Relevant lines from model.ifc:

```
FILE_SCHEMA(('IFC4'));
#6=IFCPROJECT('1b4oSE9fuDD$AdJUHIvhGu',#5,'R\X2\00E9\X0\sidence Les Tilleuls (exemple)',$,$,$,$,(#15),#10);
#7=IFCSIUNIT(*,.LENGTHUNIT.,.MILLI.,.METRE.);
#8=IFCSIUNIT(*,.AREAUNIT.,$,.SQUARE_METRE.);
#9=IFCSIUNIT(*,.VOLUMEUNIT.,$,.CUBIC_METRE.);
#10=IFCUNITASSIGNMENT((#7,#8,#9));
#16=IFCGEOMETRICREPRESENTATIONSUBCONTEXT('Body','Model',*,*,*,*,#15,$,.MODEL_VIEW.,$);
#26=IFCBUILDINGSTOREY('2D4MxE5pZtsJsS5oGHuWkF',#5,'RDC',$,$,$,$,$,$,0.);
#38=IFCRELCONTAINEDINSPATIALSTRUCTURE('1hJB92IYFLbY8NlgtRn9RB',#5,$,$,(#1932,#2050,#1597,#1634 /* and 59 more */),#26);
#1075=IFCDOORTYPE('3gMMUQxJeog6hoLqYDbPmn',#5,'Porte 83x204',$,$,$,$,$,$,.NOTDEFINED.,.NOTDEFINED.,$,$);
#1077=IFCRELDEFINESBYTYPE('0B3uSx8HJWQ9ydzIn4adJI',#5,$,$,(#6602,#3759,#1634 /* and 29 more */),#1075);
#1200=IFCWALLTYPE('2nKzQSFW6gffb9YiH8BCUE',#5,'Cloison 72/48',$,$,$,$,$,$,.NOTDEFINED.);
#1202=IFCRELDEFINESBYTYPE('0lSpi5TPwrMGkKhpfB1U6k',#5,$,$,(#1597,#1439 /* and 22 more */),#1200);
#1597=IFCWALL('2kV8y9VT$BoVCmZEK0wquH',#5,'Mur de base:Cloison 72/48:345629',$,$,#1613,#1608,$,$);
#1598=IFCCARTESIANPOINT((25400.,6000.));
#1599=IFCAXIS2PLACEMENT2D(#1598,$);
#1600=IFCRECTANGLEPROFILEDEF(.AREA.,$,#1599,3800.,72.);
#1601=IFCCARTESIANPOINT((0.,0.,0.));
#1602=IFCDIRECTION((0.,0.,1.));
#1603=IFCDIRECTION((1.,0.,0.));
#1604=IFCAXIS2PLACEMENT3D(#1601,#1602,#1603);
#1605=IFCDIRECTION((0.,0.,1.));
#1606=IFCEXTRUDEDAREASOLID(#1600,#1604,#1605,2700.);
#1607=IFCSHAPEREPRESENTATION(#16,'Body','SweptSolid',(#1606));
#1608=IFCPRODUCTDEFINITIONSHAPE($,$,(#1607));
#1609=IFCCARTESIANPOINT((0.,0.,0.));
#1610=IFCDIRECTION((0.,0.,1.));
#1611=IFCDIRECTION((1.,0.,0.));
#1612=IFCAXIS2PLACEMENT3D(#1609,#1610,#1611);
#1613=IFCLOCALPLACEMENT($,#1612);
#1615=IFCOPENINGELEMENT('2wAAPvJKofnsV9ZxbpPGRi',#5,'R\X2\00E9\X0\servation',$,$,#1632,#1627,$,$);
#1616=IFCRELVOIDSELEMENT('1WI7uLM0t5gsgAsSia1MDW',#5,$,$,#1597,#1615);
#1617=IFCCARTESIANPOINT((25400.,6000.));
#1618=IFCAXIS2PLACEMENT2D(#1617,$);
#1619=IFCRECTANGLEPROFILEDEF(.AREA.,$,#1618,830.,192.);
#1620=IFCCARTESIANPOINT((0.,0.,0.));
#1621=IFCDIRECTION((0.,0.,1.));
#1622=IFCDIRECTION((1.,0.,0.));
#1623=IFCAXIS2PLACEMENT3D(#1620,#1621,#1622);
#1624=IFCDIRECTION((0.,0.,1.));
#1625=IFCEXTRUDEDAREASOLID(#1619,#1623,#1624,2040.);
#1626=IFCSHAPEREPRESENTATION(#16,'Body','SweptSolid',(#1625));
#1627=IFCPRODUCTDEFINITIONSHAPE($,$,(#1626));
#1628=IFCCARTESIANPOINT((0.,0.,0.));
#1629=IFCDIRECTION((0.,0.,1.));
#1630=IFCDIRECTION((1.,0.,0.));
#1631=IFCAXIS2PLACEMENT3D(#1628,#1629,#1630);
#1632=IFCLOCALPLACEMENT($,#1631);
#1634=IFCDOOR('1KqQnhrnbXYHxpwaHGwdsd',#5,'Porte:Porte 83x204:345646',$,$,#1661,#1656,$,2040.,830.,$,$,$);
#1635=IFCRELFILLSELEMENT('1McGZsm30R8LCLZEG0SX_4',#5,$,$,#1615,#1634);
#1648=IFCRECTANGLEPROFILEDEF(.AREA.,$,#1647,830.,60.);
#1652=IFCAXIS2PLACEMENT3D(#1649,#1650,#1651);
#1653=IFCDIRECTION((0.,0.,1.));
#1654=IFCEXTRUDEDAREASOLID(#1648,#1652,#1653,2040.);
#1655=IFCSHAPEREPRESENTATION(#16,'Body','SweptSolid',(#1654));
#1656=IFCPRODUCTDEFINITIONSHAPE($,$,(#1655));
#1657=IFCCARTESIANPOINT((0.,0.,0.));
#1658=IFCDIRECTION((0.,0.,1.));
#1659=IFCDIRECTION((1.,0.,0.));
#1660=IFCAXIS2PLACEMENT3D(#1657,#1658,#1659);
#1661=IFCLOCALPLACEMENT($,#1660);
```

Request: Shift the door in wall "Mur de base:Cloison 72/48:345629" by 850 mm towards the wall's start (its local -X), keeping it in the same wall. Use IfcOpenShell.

```python
import ifcopenshell
import ifcopenshell.api.geometry
import ifcopenshell.util.placement
import ifcopenshell.util.unit

model = ifcopenshell.open("model.ifc")
unit_scale = ifcopenshell.util.unit.calculate_unit_scale(model)

door = model.by_id(1634)
opening = door.FillsVoids[0].RelatingOpeningElement
wall = opening.VoidsElements[0].RelatingBuildingElement

wall_matrix = ifcopenshell.util.placement.get_local_placement(wall.ObjectPlacement)
shift = wall_matrix[:3, 0] * -0.85 / unit_scale
before = ifcopenshell.util.placement.get_local_placement(door.ObjectPlacement)[:3, 3].copy()

# The door is not placed relative to its opening, so move both.
for product in (opening, door):
    matrix = ifcopenshell.util.placement.get_local_placement(product.ObjectPlacement)
    matrix[:3, 3] += shift
    ifcopenshell.api.geometry.edit_object_placement(model, product=product, matrix=matrix, is_si=False)

after = ifcopenshell.util.placement.get_local_placement(door.ObjectPlacement)[:3, 3]
print("door moved by", (after - before).round(3) + 0.0)

model.write("model_v2.ifc")
```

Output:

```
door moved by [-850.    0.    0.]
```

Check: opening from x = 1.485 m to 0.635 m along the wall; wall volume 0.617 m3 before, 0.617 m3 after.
